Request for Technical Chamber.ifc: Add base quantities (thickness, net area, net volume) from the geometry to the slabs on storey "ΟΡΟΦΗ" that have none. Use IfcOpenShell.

First a look at what the model holds.

```python
import ifcopenshell
import ifcopenshell.util.element
import ifcopenshell.util.unit

model = ifcopenshell.open("Technical Chamber.ifc")
print(model.schema)
for unit_type in ("LENGTHUNIT", "AREAUNIT", "VOLUMEUNIT"):
    print(unit_type, ifcopenshell.util.unit.calculate_unit_scale(model, unit_type))
storey = next(s for s in model.by_type("IfcBuildingStorey") if s.Name == "ΟΡΟΦΗ")
slabs = [e for e in ifcopenshell.util.element.get_decomposition(storey) if e.is_a("IfcSlab")]
for e in sorted(slabs, key=lambda e: e.id()):
    print(e.id(), e.is_a(), e.Name, list(ifcopenshell.util.element.get_psets(e, qtos_only=True)), sep=" | ")
```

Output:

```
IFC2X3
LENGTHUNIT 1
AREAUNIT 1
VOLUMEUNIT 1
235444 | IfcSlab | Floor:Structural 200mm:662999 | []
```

```python
import ifcopenshell
import ifcopenshell.api.pset
import ifcopenshell.geom
import ifcopenshell.util.element
import ifcopenshell.util.shape
import ifcopenshell.util.unit

model = ifcopenshell.open("Technical Chamber.ifc")
unit_scale = ifcopenshell.util.unit.calculate_unit_scale(model)
area_scale = ifcopenshell.util.unit.calculate_unit_scale(model, "AREAUNIT")
volume_scale = ifcopenshell.util.unit.calculate_unit_scale(model, "VOLUMEUNIT")
settings = ifcopenshell.geom.settings()

storey = next(s for s in model.by_type("IfcBuildingStorey") if s.Name == "ΟΡΟΦΗ")
slabs = [e for e in ifcopenshell.util.element.get_decomposition(storey) if e.is_a("IfcSlab")]

for e in sorted(slabs, key=lambda e: e.id()):
    if ifcopenshell.util.element.get_psets(e, qtos_only=True, should_inherit=False):
        continue
    # Geometry comes back in metres, in the element's own axes.
    shape = ifcopenshell.geom.create_shape(settings, e)
    values = {
        "Width": ifcopenshell.util.shape.get_z(shape.geometry) / unit_scale,
        "NetArea": ifcopenshell.util.shape.get_footprint_area(shape.geometry) / area_scale,
        "NetVolume": ifcopenshell.util.shape.get_volume(shape.geometry) / volume_scale,
    }
    qto = ifcopenshell.api.pset.add_qto(model, product=e, name="BaseQuantities")
    ifcopenshell.api.pset.edit_qto(model, qto=qto, properties=values)
    print(e.id(), {k: round(v, 3) for k, v in values.items()})

model.write("Technical Chamber-out.ifc")
```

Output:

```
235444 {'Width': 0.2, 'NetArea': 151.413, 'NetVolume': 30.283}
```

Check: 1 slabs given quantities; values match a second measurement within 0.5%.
